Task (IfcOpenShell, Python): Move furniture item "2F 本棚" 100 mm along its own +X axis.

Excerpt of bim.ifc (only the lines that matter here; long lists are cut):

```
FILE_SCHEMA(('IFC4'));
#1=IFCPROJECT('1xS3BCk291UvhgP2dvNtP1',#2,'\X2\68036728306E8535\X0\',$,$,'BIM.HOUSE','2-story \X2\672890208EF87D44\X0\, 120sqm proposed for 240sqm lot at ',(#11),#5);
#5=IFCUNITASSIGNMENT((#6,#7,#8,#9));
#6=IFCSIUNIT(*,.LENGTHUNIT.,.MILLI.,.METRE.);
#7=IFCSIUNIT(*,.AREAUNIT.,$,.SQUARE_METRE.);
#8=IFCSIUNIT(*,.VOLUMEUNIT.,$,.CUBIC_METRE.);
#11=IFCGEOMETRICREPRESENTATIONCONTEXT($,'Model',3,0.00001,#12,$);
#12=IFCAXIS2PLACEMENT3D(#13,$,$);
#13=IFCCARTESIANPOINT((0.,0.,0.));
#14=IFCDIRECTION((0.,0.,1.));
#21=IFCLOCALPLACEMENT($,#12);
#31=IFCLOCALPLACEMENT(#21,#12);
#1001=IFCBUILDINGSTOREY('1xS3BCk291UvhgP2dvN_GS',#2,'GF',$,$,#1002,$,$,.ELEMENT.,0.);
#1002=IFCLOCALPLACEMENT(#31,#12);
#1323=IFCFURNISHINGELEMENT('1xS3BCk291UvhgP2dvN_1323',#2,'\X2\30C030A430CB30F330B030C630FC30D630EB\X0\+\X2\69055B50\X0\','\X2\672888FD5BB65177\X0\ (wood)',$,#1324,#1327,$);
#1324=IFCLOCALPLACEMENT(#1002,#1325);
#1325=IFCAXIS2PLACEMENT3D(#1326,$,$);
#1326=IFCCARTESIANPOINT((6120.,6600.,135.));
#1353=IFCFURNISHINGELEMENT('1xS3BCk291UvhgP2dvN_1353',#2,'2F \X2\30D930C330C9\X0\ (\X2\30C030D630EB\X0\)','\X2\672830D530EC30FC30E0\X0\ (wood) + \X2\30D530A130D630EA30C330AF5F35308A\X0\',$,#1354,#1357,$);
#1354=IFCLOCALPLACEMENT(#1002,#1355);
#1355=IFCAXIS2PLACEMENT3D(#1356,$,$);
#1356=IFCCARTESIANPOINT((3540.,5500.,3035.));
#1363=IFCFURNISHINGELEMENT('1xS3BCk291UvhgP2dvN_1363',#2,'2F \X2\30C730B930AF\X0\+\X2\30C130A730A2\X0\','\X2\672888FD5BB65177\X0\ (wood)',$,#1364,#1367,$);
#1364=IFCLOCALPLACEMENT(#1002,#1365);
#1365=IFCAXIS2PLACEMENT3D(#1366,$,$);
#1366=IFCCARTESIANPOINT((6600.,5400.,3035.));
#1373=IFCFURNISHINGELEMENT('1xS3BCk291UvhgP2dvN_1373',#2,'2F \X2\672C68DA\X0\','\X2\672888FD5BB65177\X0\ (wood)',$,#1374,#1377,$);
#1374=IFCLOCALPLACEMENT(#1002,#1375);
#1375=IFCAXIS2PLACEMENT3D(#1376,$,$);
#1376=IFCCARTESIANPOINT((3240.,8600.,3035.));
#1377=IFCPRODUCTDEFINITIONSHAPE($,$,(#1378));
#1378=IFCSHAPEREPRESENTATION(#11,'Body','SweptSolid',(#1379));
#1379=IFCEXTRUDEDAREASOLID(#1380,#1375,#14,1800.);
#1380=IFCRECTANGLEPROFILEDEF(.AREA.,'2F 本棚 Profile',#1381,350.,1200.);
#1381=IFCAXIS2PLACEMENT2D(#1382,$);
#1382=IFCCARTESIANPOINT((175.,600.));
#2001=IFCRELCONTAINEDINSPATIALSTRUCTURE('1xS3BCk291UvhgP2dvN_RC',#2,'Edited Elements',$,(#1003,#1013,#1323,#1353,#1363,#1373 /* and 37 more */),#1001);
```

```python
import ifcopenshell
import ifcopenshell.api.geometry
import ifcopenshell.util.placement
import ifcopenshell.util.unit

model = ifcopenshell.open("bim.ifc")
unit_scale = ifcopenshell.util.unit.calculate_unit_scale(model)

item = model.by_guid("1xS3BCk291UvhgP2dvN_1373")
matrix = ifcopenshell.util.placement.get_local_placement(item.ObjectPlacement)
matrix[:3, 3] += matrix[:3, 0] * 0.1 / unit_scale
ifcopenshell.api.geometry.edit_object_placement(model, product=item, matrix=matrix, is_si=False)

print(ifcopenshell.util.placement.get_local_placement(item.ObjectPlacement).round(3) + 0.0)

model.write("bim_edited.ifc")
```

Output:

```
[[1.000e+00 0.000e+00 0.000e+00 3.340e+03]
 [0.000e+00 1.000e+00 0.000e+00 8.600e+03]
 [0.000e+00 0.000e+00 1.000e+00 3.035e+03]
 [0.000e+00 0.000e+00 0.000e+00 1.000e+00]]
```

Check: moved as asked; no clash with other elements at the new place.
